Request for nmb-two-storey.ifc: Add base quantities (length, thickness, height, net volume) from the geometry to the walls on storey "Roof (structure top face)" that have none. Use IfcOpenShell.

First a look at what the model holds.

```python
import ifcopenshell
import ifcopenshell.util.element
import ifcopenshell.util.unit

model = ifcopenshell.open("nmb-two-storey.ifc")
print(model.schema)
for unit_type in ("LENGTHUNIT", "AREAUNIT", "VOLUMEUNIT"):
    print(unit_type, ifcopenshell.util.unit.calculate_unit_scale(model, unit_type))
storey = next(s for s in model.by_type("IfcBuildingStorey") if s.Name == "Roof (structure top face)")
walls = [e for e in ifcopenshell.util.element.get_decomposition(storey) if e.is_a("IfcWall")]
for e in sorted(walls, key=lambda e: e.id()):
    print(e.id(), e.is_a(), e.Name, list(ifcopenshell.util.element.get_psets(e, qtos_only=True)), sep=" | ")
```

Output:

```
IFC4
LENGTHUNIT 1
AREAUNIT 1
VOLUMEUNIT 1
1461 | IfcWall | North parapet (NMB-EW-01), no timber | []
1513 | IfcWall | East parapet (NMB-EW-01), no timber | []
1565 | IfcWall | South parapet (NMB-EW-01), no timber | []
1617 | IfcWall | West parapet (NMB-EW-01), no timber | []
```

```python
import ifcopenshell
import ifcopenshell.api.pset
import ifcopenshell.geom
import ifcopenshell.util.element
import ifcopenshell.util.shape
import ifcopenshell.util.unit

model = ifcopenshell.open("nmb-two-storey.ifc")
unit_scale = ifcopenshell.util.unit.calculate_unit_scale(model)
volume_scale = ifcopenshell.util.unit.calculate_unit_scale(model, "VOLUMEUNIT")
settings = ifcopenshell.geom.settings()

storey = next(s for s in model.by_type("IfcBuildingStorey") if s.Name == "Roof (structure top face)")
walls = [e for e in ifcopenshell.util.element.get_decomposition(storey) if e.is_a("IfcWall")]

for e in sorted(walls, key=lambda e: e.id()):
    if ifcopenshell.util.element.get_psets(e, qtos_only=True, should_inherit=False):
        continue
    # Geometry comes back in metres, in the element's own axes.
    shape = ifcopenshell.geom.create_shape(settings, e)
    values = {
        "Length": ifcopenshell.util.shape.get_x(shape.geometry) / unit_scale,
        "Width": ifcopenshell.util.shape.get_y(shape.geometry) / unit_scale,
        "Height": ifcopenshell.util.shape.get_z(shape.geometry) / unit_scale,
        "NetVolume": ifcopenshell.util.shape.get_volume(shape.geometry) / volume_scale,
    }
    qto = ifcopenshell.api.pset.add_qto(model, product=e, name="Qto_WallBaseQuantities")
    ifcopenshell.api.pset.edit_qto(model, qto=qto, properties=values)
    print(e.id(), {k: round(v, 3) for k, v in values.items()})

model.write("nmb-two-storey_edited.ifc")
```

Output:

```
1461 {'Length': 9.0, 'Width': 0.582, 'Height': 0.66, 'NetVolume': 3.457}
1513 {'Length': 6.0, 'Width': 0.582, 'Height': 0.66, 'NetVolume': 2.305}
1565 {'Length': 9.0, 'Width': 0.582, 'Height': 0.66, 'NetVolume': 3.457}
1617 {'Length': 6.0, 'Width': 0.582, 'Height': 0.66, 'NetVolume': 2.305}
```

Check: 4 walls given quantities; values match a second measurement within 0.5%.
